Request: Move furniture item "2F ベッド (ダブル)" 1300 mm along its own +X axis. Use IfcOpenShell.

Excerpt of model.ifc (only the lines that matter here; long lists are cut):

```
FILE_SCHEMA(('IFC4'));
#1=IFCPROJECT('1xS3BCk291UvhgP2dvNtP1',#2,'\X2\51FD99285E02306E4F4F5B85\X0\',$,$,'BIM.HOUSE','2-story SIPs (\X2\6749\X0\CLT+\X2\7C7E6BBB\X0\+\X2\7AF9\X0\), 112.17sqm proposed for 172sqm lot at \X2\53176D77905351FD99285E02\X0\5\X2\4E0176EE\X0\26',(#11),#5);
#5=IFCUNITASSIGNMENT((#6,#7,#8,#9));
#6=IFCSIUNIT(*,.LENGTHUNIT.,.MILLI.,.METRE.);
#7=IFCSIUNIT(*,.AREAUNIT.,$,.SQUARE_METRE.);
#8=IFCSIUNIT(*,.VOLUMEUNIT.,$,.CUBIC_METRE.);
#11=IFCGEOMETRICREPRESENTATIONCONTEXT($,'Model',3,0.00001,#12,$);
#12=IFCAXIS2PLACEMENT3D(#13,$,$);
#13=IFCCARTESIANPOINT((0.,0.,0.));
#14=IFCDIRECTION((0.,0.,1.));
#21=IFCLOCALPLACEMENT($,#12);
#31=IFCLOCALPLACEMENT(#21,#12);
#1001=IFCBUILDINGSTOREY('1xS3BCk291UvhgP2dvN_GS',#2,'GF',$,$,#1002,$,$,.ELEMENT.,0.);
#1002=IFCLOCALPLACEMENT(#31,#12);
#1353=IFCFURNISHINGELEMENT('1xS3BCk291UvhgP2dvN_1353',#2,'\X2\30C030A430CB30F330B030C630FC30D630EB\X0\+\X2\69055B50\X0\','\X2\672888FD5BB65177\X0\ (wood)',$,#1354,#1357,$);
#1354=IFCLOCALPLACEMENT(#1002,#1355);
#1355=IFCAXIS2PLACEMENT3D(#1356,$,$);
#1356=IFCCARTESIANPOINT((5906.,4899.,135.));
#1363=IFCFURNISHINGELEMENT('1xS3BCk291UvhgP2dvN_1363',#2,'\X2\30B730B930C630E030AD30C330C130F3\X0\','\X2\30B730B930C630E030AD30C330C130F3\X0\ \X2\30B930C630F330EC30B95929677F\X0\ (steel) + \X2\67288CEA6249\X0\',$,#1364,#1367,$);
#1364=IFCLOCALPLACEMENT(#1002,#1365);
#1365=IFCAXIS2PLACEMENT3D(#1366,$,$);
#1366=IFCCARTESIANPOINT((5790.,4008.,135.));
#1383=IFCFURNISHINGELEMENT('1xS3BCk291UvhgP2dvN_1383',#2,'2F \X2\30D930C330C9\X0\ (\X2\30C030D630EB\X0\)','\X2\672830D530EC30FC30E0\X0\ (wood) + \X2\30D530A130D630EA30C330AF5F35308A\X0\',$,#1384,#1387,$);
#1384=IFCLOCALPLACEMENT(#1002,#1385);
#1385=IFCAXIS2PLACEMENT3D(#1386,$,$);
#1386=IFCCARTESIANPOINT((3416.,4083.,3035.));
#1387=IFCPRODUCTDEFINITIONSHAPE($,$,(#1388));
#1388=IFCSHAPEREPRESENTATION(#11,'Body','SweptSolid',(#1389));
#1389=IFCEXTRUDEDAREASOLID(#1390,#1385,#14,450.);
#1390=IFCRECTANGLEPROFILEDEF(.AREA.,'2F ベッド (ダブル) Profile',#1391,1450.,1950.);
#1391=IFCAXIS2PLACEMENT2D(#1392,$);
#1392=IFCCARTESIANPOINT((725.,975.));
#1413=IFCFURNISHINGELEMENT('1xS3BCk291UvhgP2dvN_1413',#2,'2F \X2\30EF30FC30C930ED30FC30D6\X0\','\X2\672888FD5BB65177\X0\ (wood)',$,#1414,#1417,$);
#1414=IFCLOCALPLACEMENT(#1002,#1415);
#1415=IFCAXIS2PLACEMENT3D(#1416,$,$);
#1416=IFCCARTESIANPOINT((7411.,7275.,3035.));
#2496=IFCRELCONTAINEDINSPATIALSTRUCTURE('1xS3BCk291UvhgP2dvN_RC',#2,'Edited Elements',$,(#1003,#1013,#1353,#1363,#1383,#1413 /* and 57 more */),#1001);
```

```python
import ifcopenshell
import ifcopenshell.api.geometry
import ifcopenshell.util.placement

model = ifcopenshell.open("model.ifc")

item = model.by_id(1383)
matrix = ifcopenshell.util.placement.get_local_placement(item.ObjectPlacement)
matrix[:3, 3] += matrix[:3, 0] * 1300.0
ifcopenshell.api.geometry.edit_object_placement(model, product=item, matrix=matrix, is_si=False)

print(ifcopenshell.util.placement.get_local_placement(item.ObjectPlacement).round(3) + 0.0)

model.write("model_edited.ifc")
```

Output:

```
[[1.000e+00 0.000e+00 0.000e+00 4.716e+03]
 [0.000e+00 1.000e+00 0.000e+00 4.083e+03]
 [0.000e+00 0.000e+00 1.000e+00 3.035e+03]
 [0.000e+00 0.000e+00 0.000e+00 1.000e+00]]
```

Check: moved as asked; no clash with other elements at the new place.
